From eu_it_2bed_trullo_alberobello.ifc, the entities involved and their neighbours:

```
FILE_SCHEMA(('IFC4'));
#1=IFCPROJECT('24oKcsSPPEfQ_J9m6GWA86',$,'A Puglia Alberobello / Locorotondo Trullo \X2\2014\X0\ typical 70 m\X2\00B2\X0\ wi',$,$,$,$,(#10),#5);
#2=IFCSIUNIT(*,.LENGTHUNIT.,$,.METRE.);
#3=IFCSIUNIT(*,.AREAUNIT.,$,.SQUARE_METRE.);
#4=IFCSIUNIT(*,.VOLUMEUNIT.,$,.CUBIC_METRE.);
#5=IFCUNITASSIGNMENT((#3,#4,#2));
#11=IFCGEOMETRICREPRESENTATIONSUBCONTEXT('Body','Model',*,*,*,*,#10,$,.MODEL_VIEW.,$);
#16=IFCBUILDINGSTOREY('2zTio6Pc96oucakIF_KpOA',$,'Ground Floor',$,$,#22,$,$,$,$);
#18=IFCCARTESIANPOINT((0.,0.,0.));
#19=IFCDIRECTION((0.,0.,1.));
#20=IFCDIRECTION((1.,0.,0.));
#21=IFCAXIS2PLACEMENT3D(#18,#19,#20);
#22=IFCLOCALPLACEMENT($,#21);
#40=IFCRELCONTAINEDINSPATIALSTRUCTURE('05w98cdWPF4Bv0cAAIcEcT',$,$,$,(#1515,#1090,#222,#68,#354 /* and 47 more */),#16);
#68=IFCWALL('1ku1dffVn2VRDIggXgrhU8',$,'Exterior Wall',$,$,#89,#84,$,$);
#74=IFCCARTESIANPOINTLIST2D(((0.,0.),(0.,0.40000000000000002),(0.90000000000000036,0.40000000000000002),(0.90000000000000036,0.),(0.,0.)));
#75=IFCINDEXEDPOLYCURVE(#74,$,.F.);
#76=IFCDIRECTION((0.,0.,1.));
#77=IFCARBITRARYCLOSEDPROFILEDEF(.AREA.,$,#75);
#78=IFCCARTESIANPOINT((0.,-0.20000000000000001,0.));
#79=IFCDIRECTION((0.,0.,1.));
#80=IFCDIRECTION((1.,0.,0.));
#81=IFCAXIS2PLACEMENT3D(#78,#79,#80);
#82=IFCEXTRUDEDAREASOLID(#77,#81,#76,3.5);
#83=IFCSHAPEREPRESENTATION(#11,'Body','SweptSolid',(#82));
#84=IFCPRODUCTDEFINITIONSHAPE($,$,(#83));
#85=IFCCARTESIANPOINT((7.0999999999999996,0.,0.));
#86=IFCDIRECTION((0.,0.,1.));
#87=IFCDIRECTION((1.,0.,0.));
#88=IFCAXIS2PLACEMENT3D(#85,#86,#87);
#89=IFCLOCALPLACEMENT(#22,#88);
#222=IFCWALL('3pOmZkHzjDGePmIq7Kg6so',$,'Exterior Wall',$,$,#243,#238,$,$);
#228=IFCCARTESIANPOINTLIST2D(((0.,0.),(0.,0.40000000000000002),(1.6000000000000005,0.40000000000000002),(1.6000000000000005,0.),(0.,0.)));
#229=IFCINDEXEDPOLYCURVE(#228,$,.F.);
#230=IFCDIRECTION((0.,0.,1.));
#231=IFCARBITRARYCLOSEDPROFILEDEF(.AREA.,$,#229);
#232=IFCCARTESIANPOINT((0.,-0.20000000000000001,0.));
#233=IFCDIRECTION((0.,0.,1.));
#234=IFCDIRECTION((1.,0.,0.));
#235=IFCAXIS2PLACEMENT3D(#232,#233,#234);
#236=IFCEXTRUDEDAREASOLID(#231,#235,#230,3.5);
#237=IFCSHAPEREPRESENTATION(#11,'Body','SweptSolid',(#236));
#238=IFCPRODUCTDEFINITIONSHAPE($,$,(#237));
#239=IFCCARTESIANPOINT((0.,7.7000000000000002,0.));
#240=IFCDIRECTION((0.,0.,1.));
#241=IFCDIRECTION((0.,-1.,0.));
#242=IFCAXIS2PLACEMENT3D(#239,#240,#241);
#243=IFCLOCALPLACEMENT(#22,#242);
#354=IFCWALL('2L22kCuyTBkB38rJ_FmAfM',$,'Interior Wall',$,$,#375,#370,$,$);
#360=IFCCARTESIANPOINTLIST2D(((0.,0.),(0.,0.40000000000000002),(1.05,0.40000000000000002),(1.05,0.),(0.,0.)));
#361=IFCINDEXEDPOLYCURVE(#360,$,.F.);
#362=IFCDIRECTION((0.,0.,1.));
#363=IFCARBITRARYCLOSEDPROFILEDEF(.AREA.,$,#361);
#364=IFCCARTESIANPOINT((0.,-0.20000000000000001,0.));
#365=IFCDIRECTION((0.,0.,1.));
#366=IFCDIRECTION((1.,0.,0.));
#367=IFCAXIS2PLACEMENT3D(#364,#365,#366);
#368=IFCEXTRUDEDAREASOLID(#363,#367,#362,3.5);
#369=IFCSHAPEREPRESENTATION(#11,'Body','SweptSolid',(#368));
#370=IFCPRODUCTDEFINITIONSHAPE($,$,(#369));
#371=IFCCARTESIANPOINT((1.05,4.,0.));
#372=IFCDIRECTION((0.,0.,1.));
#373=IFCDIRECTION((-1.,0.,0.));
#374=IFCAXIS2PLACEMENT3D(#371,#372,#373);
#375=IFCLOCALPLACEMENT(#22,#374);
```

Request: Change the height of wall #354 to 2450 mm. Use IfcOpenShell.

```python
import ifcopenshell
import ifcopenshell.geom
import ifcopenshell.util.representation
import ifcopenshell.util.shape

model = ifcopenshell.open("eu_it_2bed_trullo_alberobello.ifc")
settings = ifcopenshell.geom.settings()


def volume(element):
    """Net volume in cubic metres, openings subtracted."""
    shape = ifcopenshell.geom.create_shape(settings, element)
    return ifcopenshell.util.shape.get_volume(shape.geometry)


wall = model.by_id(354)
before = volume(wall)

body = ifcopenshell.util.representation.get_representation(wall, "Model", "Body")
solid = body.Items[0]
old_height = solid.Depth
solid.Depth = 2.45
after = volume(wall)

print(f"height {old_height:g} -> {solid.Depth:g}, volume {before:.3f} -> {after:.3f} m3")

model.write("eu_it_2bed_trullo_alberobello_updated.ifc")
```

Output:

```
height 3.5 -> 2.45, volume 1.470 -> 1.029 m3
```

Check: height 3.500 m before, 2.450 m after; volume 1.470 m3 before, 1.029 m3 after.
